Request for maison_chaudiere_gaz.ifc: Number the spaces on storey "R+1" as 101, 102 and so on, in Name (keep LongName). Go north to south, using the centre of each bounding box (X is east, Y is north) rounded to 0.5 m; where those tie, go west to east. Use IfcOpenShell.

First a look at what the model holds.

```python
import ifcopenshell
import ifcopenshell.util.element
import ifcopenshell.util.placement

model = ifcopenshell.open("maison_chaudiere_gaz.ifc")
print(model.schema)
storey = next(s for s in model.by_type("IfcBuildingStorey") if s.Name == "R+1")
spaces = [e for e in ifcopenshell.util.element.get_decomposition(storey) if e.is_a("IfcSpace")]
for e in sorted(spaces, key=lambda e: e.id()):
    origin = ifcopenshell.util.placement.get_local_placement(e.ObjectPlacement)[:3, 3]
    print(e.id(), e.Name, e.LongName, origin.round(2) + 0.0, sep=" | ")
```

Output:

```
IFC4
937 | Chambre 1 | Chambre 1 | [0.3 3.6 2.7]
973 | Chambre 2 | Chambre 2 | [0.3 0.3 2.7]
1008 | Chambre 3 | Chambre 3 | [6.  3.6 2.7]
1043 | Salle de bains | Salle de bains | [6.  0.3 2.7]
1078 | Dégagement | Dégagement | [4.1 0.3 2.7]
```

```python
import ifcopenshell
import ifcopenshell.geom
import ifcopenshell.util.element
import ifcopenshell.util.shape

model = ifcopenshell.open("maison_chaudiere_gaz.ifc")
settings = ifcopenshell.geom.settings()
settings.set("use-world-coords", True)


def centre(element):
    shape = ifcopenshell.geom.create_shape(settings, element)
    return ifcopenshell.util.shape.get_bbox_centroid(shape.geometry)


storey = next(s for s in model.by_type("IfcBuildingStorey") if s.Name == "R+1")
spaces = [e for e in ifcopenshell.util.element.get_decomposition(storey) if e.is_a("IfcSpace")]

# Insertion points can sit at a corner or the storey origin, so sort by the geometry (in metres).
centres = {e: centre(e) for e in spaces}
spaces.sort(key=lambda e: (-round(centres[e][1] / 0.5), centres[e][0]))

for i, e in enumerate(spaces, start=1):
    number = f"1{i:02d}"
    e.Name = number
    print(e.id(), number)

model.write("maison_chaudiere_gaz_edited.ifc")
```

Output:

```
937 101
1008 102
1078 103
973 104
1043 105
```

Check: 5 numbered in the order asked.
